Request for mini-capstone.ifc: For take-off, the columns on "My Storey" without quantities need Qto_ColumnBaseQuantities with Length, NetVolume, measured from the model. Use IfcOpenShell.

First a look at what the model holds.

```python
import ifcopenshell
import ifcopenshell.util.element
import ifcopenshell.util.unit

model = ifcopenshell.open("mini-capstone.ifc")
print(model.schema)
for unit_type in ("LENGTHUNIT", "AREAUNIT", "VOLUMEUNIT"):
    print(unit_type, ifcopenshell.util.unit.calculate_unit_scale(model, unit_type))
storey = next(s for s in model.by_type("IfcBuildingStorey") if s.Name == "My Storey")
columns = [e for e in ifcopenshell.util.element.get_decomposition(storey) if e.is_a("IfcColumn")]
for e in sorted(columns, key=lambda e: e.id()):
    print(e.id(), e.is_a(), e.Name, list(ifcopenshell.util.element.get_psets(e, qtos_only=True)), sep=" | ")
```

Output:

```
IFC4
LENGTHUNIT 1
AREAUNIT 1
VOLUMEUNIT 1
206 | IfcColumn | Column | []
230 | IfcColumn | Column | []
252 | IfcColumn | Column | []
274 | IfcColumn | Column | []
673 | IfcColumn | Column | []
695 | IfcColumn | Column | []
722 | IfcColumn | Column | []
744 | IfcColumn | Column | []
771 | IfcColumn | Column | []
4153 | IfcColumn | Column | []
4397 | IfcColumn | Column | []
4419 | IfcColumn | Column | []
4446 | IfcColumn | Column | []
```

```python
import ifcopenshell
import ifcopenshell.api.pset
import ifcopenshell.geom
import ifcopenshell.util.element
import ifcopenshell.util.shape
import ifcopenshell.util.unit

model = ifcopenshell.open("mini-capstone.ifc")
unit_scale = ifcopenshell.util.unit.calculate_unit_scale(model)
volume_scale = ifcopenshell.util.unit.calculate_unit_scale(model, "VOLUMEUNIT")
settings = ifcopenshell.geom.settings()

storey = next(s for s in model.by_type("IfcBuildingStorey") if s.Name == "My Storey")
columns = [e for e in ifcopenshell.util.element.get_decomposition(storey) if e.is_a("IfcColumn")]

for e in sorted(columns, key=lambda e: e.id()):
    if ifcopenshell.util.element.get_psets(e, qtos_only=True, should_inherit=False):
        continue
    # Geometry comes back in metres, in the element's own axes.
    shape = ifcopenshell.geom.create_shape(settings, e)
    values = {
        "Length": ifcopenshell.util.shape.get_z(shape.geometry) / unit_scale,
        "NetVolume": ifcopenshell.util.shape.get_volume(shape.geometry) / volume_scale,
    }
    qto = ifcopenshell.api.pset.add_qto(model, product=e, name="Qto_ColumnBaseQuantities")
    ifcopenshell.api.pset.edit_qto(model, qto=qto, properties=values)
    print(e.id(), {k: round(v, 3) for k, v in values.items()})

model.write("mini-capstone_edited.ifc")
```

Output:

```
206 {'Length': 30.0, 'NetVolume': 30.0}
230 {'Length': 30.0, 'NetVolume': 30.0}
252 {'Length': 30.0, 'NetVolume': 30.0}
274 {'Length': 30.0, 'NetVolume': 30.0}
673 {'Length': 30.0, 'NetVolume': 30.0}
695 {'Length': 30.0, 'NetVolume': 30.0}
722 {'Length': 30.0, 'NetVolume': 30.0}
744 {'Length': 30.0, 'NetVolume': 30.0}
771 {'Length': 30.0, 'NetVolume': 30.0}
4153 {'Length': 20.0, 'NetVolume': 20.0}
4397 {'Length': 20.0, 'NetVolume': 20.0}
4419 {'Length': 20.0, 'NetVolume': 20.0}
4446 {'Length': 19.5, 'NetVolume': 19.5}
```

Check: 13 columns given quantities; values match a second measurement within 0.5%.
